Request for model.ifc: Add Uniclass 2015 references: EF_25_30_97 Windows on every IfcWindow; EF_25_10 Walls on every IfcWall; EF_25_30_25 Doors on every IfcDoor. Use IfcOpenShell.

First a look at what the model holds.

```python
import ifcopenshell

model = ifcopenshell.open("model.ifc")
print(model.schema)
print("classifications:", [c.Name for c in model.by_type("IfcClassification")])
for ifc_class in ("IfcDoor", "IfcRoof", "IfcStair", "IfcWall", "IfcWindow"):
    print(ifc_class, len(model.by_type(ifc_class)))
```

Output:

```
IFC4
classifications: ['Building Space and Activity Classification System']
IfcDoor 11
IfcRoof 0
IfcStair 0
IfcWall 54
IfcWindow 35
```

```python
import ifcopenshell
import ifcopenshell.api.classification

model = ifcopenshell.open("model.ifc")

system = ifcopenshell.api.classification.add_classification(model, classification="Uniclass 2015")

codes = {
    "IfcWindow": ("EF_25_30_97", "Windows"),
    "IfcWall": ("EF_25_10", "Walls"),
    "IfcDoor": ("EF_25_30_25", "Doors"),
}
for ifc_class, (code, name) in codes.items():
    products = model.by_type(ifc_class)
    ifcopenshell.api.classification.add_reference(
        model, products=products, classification=system, identification=code, name=name
    )
    print(code, len(products))

model.write("model_updated.ifc")
```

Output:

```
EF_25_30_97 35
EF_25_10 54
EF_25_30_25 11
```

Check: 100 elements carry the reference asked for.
